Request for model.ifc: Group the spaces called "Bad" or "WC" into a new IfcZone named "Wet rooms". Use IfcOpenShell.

First a look at what the model holds.

```python
import ifcopenshell

model = ifcopenshell.open("model.ifc")
print(model.schema)
seen = {}
for space in model.by_type("IfcSpace"):
    seen[space.LongName] = seen.get(space.LongName, 0) + 1
for name, count in sorted(seen.items(), key=str):
    print(count, "x", name)
print("zones:", [z.Name for z in model.by_type("IfcZone")][:20])
```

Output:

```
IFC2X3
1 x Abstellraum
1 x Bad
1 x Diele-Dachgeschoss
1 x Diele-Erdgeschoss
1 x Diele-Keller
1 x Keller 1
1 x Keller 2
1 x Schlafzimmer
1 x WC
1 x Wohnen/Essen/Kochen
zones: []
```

```python
import ifcopenshell
import ifcopenshell.api.group
import ifcopenshell.api.root

model = ifcopenshell.open("model.ifc")

names = {"Bad", "WC"}
spaces = [s for s in model.by_type("IfcSpace") if s.LongName in names]

zone = ifcopenshell.api.root.create_entity(model, ifc_class="IfcZone", name="Wet rooms")
ifcopenshell.api.group.assign_group(model, products=spaces, group=zone)
print(len(spaces), "spaces in", zone.Name)

model.write("model_updated.ifc")
```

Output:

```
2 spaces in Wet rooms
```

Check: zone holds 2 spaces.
